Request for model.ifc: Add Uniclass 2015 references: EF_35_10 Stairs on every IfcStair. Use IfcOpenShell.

First a look at what the model holds.

```python
import ifcopenshell

model = ifcopenshell.open("model.ifc")
print(model.schema)
print("classifications:", [c.Name for c in model.by_type("IfcClassification")])
for ifc_class in ("IfcDoor", "IfcRoof", "IfcStair", "IfcWall", "IfcWindow"):
    print(ifc_class, len(model.by_type(ifc_class)))
```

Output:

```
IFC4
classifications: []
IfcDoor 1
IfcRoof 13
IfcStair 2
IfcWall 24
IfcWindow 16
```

```python
import ifcopenshell
import ifcopenshell.api.classification

model = ifcopenshell.open("model.ifc")

system = ifcopenshell.api.classification.add_classification(model, classification="Uniclass 2015")

codes = {
    "IfcStair": ("EF_35_10", "Stairs"),
}
for ifc_class, (code, name) in codes.items():
    products = model.by_type(ifc_class)
    ifcopenshell.api.classification.add_reference(
        model, products=products, classification=system, identification=code, name=name
    )
    print(code, len(products))

model.write("model_edited.ifc")
```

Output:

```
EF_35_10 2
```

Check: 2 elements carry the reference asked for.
